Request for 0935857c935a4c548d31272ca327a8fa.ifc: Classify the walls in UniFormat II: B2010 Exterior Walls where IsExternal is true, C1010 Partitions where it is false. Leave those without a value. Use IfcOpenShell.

First a look at what the model holds.

```python
import ifcopenshell
import ifcopenshell.util.element

model = ifcopenshell.open("0935857c935a4c548d31272ca327a8fa.ifc")
print(model.schema)
print("classifications:", [c.Name for c in model.by_type("IfcClassification")])
values = [ifcopenshell.util.element.get_pset(e, "Pset_WallCommon", "IsExternal") for e in model.by_type("IfcWall")]
for value in (True, False, None):
    print("IsExternal", value, values.count(value))
```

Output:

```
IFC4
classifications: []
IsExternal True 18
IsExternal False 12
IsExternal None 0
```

```python
import ifcopenshell
import ifcopenshell.api.classification
import ifcopenshell.util.element

model = ifcopenshell.open("0935857c935a4c548d31272ca327a8fa.ifc")

system = ifcopenshell.api.classification.add_classification(model, classification="UniFormat II")

walls = model.by_type("IfcWall")
external = {e: ifcopenshell.util.element.get_pset(e, "Pset_WallCommon", "IsExternal") for e in walls}
for flag, code, name in ((True, "B2010", "Exterior Walls"), (False, "C1010", "Partitions")):
    products = [e for e in walls if external[e] is flag]
    ifcopenshell.api.classification.add_reference(
        model, products=products, classification=system, identification=code, name=name
    )
    print(code, len(products))

model.write("0935857c935a4c548d31272ca327a8fa_updated.ifc")
```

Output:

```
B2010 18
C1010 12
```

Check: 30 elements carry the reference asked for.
